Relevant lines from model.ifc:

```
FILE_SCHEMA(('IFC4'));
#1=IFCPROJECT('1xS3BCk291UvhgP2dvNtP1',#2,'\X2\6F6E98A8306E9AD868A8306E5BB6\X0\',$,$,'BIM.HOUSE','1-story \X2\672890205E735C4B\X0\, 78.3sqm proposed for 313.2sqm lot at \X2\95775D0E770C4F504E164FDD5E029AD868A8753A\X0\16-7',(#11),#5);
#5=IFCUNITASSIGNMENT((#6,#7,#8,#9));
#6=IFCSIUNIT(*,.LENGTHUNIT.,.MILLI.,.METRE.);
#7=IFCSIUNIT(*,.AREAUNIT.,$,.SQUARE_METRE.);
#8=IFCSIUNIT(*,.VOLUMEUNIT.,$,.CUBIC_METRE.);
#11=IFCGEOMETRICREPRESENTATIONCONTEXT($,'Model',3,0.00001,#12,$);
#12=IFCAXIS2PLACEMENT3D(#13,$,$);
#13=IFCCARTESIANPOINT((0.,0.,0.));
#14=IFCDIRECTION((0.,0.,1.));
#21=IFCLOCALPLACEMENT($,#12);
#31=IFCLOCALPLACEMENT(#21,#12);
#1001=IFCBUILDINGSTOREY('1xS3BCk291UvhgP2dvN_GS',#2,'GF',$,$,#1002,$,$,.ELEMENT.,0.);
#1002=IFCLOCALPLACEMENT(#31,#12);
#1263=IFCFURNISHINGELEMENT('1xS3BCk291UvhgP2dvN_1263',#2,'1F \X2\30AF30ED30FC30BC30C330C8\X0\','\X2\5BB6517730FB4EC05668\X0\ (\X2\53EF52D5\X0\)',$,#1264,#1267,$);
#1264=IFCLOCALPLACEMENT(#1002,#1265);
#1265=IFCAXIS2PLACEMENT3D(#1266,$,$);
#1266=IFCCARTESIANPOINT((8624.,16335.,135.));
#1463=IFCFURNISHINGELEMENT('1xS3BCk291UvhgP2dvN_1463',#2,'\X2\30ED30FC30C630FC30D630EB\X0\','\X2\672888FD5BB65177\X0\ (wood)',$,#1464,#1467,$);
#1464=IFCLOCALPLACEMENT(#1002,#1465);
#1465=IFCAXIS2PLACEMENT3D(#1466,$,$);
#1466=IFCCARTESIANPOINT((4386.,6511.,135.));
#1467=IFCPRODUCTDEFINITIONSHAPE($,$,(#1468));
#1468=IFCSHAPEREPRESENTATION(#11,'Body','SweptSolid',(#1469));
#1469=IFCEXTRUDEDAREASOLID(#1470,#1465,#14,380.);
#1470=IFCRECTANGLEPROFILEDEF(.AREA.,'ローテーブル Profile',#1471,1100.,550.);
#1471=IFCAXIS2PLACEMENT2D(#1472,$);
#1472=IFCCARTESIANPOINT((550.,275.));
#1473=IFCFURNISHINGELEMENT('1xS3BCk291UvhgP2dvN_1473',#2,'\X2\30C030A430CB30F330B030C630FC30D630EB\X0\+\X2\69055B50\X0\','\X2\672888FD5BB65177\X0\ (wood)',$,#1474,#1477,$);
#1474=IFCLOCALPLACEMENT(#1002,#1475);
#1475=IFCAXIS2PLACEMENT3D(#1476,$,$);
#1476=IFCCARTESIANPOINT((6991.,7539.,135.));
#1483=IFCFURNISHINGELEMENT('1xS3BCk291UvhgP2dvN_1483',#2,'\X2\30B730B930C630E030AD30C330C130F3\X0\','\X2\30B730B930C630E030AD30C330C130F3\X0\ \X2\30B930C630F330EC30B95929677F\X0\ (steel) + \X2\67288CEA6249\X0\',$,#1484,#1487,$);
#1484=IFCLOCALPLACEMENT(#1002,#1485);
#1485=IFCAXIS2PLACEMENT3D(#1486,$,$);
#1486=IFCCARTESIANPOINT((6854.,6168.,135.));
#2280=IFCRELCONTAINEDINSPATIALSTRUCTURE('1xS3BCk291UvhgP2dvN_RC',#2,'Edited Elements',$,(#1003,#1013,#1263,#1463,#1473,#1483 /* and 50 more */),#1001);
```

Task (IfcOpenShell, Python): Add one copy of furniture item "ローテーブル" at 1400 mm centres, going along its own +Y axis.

```python
import ifcopenshell
import ifcopenshell.api.geometry
import ifcopenshell.api.root
import ifcopenshell.util.element
import ifcopenshell.util.placement

model = ifcopenshell.open("model.ifc")


def reuse_history(source, copy):
    """copy_class also copies each property set's owner history, people and application; keep the originals."""
    for rel in copy.IsDefinedBy:
        if rel.is_a("IfcRelDefinesByProperties") and (history := rel.RelatingPropertyDefinition.OwnerHistory):
            rel.RelatingPropertyDefinition.OwnerHistory = source.OwnerHistory
            ifcopenshell.util.element.remove_deep2(model, history)


source = model.by_guid("1xS3BCk291UvhgP2dvN_1463")
base = ifcopenshell.util.placement.get_local_placement(source.ObjectPlacement)
step = base[:3, 1] * 1400.0

for i in range(1, 2):
    copy = ifcopenshell.api.root.copy_class(model, product=source)
    copy.Representation = ifcopenshell.util.element.copy_deep(
        model, source.Representation, exclude=["IfcGeometricRepresentationContext", "IfcRepresentationMap"]
    )
    reuse_history(source, copy)
    matrix = base.copy()
    matrix[:3, 3] += i * step
    print("added at", matrix[:3, 3].round(3) + 0.0)
    ifcopenshell.api.geometry.edit_object_placement(model, product=copy, matrix=matrix, is_si=False)

model.write("model_rev.ifc")
```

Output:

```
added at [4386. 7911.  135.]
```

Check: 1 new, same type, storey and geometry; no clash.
